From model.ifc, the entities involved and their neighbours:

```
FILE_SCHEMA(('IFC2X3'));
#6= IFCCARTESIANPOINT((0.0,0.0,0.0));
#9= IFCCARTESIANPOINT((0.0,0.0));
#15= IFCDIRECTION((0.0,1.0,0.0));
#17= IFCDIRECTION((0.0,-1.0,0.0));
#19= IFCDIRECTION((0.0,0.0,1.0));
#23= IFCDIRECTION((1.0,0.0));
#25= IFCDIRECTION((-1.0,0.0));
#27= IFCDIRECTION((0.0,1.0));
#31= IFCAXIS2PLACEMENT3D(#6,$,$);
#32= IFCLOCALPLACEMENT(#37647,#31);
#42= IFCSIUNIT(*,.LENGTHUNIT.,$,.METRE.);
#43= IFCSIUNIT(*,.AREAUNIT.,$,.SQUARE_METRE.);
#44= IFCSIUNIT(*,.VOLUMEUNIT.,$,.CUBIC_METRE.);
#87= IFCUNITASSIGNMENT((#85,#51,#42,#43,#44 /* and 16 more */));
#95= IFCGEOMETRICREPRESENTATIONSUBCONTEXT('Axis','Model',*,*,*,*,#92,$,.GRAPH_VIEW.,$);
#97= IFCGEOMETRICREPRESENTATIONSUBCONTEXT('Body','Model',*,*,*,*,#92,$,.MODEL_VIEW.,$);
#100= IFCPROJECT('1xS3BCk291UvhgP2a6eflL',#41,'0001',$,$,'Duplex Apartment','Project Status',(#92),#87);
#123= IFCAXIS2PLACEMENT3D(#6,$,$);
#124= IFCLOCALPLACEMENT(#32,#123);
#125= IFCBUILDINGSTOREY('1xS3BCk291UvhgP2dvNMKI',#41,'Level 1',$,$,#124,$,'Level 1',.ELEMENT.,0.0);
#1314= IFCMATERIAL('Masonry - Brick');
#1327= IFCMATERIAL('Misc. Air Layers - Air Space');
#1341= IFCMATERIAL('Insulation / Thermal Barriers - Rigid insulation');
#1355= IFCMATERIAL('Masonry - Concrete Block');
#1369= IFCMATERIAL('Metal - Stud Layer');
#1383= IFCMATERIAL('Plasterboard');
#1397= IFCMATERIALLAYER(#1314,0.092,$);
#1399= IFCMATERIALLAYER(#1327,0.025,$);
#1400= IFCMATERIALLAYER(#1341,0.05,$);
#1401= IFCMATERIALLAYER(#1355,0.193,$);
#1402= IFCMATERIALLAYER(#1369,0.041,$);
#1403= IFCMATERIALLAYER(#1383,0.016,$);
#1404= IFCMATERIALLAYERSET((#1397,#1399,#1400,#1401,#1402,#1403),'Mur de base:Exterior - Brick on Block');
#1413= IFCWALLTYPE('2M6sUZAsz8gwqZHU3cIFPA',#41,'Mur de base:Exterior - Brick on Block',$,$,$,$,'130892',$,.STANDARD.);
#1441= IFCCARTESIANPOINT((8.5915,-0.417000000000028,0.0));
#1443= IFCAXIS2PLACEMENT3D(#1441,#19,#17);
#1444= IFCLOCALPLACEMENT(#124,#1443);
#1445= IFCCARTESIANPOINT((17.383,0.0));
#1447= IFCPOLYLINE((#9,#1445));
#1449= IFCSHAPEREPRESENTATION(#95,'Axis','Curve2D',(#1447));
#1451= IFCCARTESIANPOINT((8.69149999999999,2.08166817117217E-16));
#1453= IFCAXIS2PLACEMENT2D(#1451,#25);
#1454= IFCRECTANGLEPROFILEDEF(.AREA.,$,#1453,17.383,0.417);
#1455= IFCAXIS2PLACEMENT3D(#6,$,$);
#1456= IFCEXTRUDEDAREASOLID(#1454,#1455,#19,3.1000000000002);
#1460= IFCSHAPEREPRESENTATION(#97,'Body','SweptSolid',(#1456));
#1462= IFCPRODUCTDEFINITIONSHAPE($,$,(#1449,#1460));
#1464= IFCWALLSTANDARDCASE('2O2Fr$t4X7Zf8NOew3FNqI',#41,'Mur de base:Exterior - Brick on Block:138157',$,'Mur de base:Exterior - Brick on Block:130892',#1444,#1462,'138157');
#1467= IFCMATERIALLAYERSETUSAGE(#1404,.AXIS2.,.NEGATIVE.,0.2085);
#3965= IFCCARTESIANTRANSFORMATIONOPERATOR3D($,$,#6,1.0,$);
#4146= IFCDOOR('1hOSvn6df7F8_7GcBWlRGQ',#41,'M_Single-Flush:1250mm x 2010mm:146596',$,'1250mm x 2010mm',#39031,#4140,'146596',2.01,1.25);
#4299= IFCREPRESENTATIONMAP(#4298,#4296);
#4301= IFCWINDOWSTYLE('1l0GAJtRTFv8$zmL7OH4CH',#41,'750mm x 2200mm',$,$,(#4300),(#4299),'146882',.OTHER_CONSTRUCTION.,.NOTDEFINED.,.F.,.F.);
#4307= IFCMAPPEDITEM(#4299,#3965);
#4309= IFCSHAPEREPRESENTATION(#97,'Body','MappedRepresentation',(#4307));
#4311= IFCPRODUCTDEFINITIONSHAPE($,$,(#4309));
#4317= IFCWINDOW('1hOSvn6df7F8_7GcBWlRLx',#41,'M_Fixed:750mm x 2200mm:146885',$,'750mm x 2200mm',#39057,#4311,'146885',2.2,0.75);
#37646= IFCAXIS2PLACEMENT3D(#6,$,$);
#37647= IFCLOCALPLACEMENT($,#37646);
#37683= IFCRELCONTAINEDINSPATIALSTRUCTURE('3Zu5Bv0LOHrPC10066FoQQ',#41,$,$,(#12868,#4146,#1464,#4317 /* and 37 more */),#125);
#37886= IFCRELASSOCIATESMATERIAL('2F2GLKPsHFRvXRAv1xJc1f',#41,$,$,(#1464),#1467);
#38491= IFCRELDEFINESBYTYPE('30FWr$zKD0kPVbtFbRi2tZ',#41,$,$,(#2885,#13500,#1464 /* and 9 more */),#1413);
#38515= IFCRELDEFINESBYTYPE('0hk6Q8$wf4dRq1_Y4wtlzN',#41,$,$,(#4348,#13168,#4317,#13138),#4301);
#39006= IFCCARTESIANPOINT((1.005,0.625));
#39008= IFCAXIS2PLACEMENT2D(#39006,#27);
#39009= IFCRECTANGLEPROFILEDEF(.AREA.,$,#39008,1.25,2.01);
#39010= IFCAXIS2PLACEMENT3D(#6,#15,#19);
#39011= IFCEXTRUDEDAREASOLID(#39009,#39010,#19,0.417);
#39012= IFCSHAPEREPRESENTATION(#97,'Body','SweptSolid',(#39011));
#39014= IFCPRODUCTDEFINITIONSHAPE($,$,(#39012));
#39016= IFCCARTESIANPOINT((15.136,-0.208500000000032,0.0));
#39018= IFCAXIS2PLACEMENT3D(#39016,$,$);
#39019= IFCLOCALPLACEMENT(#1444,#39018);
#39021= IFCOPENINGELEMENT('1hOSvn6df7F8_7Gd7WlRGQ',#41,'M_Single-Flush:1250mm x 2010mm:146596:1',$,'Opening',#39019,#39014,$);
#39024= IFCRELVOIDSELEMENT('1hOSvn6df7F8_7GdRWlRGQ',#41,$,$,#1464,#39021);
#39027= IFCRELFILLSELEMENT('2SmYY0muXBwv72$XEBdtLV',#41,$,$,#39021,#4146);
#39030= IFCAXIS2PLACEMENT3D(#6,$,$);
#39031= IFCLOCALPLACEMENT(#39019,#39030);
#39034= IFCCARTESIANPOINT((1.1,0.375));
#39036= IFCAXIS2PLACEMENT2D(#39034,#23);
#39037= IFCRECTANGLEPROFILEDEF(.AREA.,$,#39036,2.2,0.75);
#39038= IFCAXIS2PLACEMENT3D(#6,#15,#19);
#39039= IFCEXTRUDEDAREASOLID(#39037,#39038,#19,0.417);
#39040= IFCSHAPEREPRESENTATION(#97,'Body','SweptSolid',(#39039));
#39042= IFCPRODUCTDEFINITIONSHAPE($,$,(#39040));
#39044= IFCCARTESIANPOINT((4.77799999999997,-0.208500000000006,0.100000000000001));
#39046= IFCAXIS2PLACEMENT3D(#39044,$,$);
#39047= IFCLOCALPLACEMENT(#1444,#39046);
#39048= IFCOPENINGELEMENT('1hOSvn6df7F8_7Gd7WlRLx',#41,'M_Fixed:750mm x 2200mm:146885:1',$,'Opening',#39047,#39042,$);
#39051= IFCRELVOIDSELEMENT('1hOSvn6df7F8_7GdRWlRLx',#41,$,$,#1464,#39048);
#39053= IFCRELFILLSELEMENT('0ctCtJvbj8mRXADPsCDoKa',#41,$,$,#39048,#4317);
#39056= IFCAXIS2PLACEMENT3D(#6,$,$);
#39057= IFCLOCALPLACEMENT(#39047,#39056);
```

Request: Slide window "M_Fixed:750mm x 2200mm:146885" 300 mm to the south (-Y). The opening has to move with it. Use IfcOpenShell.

```python
import ifcopenshell
import ifcopenshell.api.geometry
import ifcopenshell.util.placement
import ifcopenshell.util.unit

model = ifcopenshell.open("model.ifc")
unit_scale = ifcopenshell.util.unit.calculate_unit_scale(model)

window = model.by_id(4317)
opening = window.FillsVoids[0].RelatingOpeningElement
wall = opening.VoidsElements[0].RelatingBuildingElement

wall_matrix = ifcopenshell.util.placement.get_local_placement(wall.ObjectPlacement)
shift = wall_matrix[:3, 0] * 0.3 / unit_scale
before = ifcopenshell.util.placement.get_local_placement(window.ObjectPlacement)[:3, 3].copy()

# The window is placed relative to its opening, so it follows when the opening moves.
matrix = ifcopenshell.util.placement.get_local_placement(opening.ObjectPlacement)
matrix[:3, 3] += shift
ifcopenshell.api.geometry.edit_object_placement(
    model, product=opening, matrix=matrix, is_si=False, should_transform_children=True
)

after = ifcopenshell.util.placement.get_local_placement(window.ObjectPlacement)[:3, 3]
print("window moved by", (after - before).round(3) + 0.0)

model.write("model_updated.ifc")
```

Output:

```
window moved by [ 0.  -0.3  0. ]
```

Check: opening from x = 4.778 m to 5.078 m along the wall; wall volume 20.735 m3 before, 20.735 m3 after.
